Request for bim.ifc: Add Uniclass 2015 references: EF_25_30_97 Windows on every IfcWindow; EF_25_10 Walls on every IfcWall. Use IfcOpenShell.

First a look at what the model holds.

```python
import ifcopenshell

model = ifcopenshell.open("bim.ifc")
print(model.schema)
print("classifications:", [c.Name for c in model.by_type("IfcClassification")])
for ifc_class in ("IfcDoor", "IfcRoof", "IfcStair", "IfcWall", "IfcWindow"):
    print(ifc_class, len(model.by_type(ifc_class)))
```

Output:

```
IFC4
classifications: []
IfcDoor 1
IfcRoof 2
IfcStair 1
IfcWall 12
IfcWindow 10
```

```python
import ifcopenshell
import ifcopenshell.api.classification

model = ifcopenshell.open("bim.ifc")

system = ifcopenshell.api.classification.add_classification(model, classification="Uniclass 2015")

codes = {
    "IfcWindow": ("EF_25_30_97", "Windows"),
    "IfcWall": ("EF_25_10", "Walls"),
}
for ifc_class, (code, name) in codes.items():
    products = model.by_type(ifc_class)
    ifcopenshell.api.classification.add_reference(
        model, products=products, classification=system, identification=code, name=name
    )
    print(code, len(products))

model.write("bim-out.ifc")
```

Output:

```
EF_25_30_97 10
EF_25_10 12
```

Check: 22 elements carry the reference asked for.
